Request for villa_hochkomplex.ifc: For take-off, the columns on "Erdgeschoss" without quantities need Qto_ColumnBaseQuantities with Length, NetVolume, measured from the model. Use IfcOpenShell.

First a look at what the model holds.

```python
import ifcopenshell
import ifcopenshell.util.element
import ifcopenshell.util.unit

model = ifcopenshell.open("villa_hochkomplex.ifc")
print(model.schema)
for unit_type in ("LENGTHUNIT", "AREAUNIT", "VOLUMEUNIT"):
    print(unit_type, ifcopenshell.util.unit.calculate_unit_scale(model, unit_type))
storey = next(s for s in model.by_type("IfcBuildingStorey") if s.Name == "Erdgeschoss")
columns = [e for e in ifcopenshell.util.element.get_decomposition(storey) if e.is_a("IfcColumn")]
for e in sorted(columns, key=lambda e: e.id()):
    print(e.id(), e.is_a(), e.Name, list(ifcopenshell.util.element.get_psets(e, qtos_only=True)), sep=" | ")
```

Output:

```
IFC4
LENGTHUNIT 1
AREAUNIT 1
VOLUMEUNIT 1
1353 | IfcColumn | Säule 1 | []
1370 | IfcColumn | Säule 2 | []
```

```python
import ifcopenshell
import ifcopenshell.api.pset
import ifcopenshell.geom
import ifcopenshell.util.element
import ifcopenshell.util.shape
import ifcopenshell.util.unit

model = ifcopenshell.open("villa_hochkomplex.ifc")
unit_scale = ifcopenshell.util.unit.calculate_unit_scale(model)
volume_scale = ifcopenshell.util.unit.calculate_unit_scale(model, "VOLUMEUNIT")
settings = ifcopenshell.geom.settings()

storey = next(s for s in model.by_type("IfcBuildingStorey") if s.Name == "Erdgeschoss")
columns = [e for e in ifcopenshell.util.element.get_decomposition(storey) if e.is_a("IfcColumn")]

for e in sorted(columns, key=lambda e: e.id()):
    if ifcopenshell.util.element.get_psets(e, qtos_only=True, should_inherit=False):
        continue
    # Geometry comes back in metres, in the element's own axes.
    shape = ifcopenshell.geom.create_shape(settings, e)
    values = {
        "Length": ifcopenshell.util.shape.get_z(shape.geometry) / unit_scale,
        "NetVolume": ifcopenshell.util.shape.get_volume(shape.geometry) / volume_scale,
    }
    qto = ifcopenshell.api.pset.add_qto(model, product=e, name="Qto_ColumnBaseQuantities")
    ifcopenshell.api.pset.edit_qto(model, qto=qto, properties=values)
    print(e.id(), {k: round(v, 3) for k, v in values.items()})

model.write("villa_hochkomplex_edited.ifc")
```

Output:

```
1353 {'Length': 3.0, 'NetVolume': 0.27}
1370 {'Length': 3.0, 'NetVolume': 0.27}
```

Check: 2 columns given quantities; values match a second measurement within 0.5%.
